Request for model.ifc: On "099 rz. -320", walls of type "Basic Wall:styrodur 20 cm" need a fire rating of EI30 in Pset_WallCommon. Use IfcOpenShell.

First a look at what the model holds.

```python
import ifcopenshell
import ifcopenshell.util.element

model = ifcopenshell.open("model.ifc")
print(model.schema)
storey = next(s for s in model.by_type("IfcBuildingStorey") if s.Name == "099 rz. -320")
walls = [e for e in ifcopenshell.util.element.get_decomposition(storey) if e.is_a("IfcWall")]
seen = {}
for e in walls:
    element_type = ifcopenshell.util.element.get_type(e)
    key = (element_type.Name if element_type != e and element_type else None, ifcopenshell.util.element.get_pset(e, "Pset_WallCommon", "FireRating"))
    seen[key] = seen.get(key, 0) + 1
for (name, value), count in sorted(seen.items(), key=str):
    print(count, "x", name, "|", value)
```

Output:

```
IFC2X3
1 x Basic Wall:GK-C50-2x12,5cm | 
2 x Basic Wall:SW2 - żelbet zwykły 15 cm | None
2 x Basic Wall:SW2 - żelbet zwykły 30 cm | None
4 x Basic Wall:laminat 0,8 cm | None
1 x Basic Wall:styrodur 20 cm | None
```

```python
import ifcopenshell
import ifcopenshell.api.pset
import ifcopenshell.util.element

model = ifcopenshell.open("model.ifc")

storey = next(s for s in model.by_type("IfcBuildingStorey") if s.Name == "099 rz. -320")
walls = [e for e in ifcopenshell.util.element.get_decomposition(storey) if e.is_a("IfcWall")]

count = 0
for e in walls:
    element_type = ifcopenshell.util.element.get_type(e)
    if element_type in (None, e) or element_type.Name != "Basic Wall:styrodur 20 cm":
        continue
    # add_pset returns the element's existing set when there is one.
    pset = ifcopenshell.api.pset.add_pset(model, product=e, name="Pset_WallCommon")
    ifcopenshell.api.pset.edit_pset(model, pset=pset, properties={"FireRating": "EI30"})
    count += 1

print(count, "walls updated")

model.write("model-out.ifc")
```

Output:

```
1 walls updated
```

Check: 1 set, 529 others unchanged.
